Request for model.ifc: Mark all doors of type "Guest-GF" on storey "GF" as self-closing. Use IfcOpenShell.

First a look at what the model holds.

```python
import ifcopenshell
import ifcopenshell.util.element

model = ifcopenshell.open("model.ifc")
print(model.schema)
storey = next(s for s in model.by_type("IfcBuildingStorey") if s.Name == "GF")
doors = [e for e in ifcopenshell.util.element.get_decomposition(storey) if e.is_a("IfcDoor")]
seen = {}
for e in doors:
    element_type = ifcopenshell.util.element.get_type(e)
    key = (element_type.Name if element_type != e and element_type else None, ifcopenshell.util.element.get_pset(e, "Pset_DoorCommon", "SelfClosing"))
    seen[key] = seen.get(key, 0) + 1
for (name, value), count in sorted(seen.items(), key=str):
    print(count, "x", name, "|", value)
```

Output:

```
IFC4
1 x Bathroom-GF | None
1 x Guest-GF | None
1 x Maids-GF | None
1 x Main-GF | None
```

```python
import ifcopenshell
import ifcopenshell.api.pset
import ifcopenshell.util.element

model = ifcopenshell.open("model.ifc")

storey = next(s for s in model.by_type("IfcBuildingStorey") if s.Name == "GF")
doors = [e for e in ifcopenshell.util.element.get_decomposition(storey) if e.is_a("IfcDoor")]

count = 0
for e in doors:
    element_type = ifcopenshell.util.element.get_type(e)
    if element_type in (None, e) or element_type.Name != "Guest-GF":
        continue
    # add_pset returns the element's existing set when there is one.
    pset = ifcopenshell.api.pset.add_pset(model, product=e, name="Pset_DoorCommon")
    ifcopenshell.api.pset.edit_pset(model, pset=pset, properties={"SelfClosing": True})
    count += 1

print(count, "doors updated")

model.write("model_edited.ifc")
```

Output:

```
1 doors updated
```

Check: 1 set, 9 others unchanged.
